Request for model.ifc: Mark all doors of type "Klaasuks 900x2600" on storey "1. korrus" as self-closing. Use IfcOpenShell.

First a look at what the model holds.

```python
import ifcopenshell
import ifcopenshell.util.element

model = ifcopenshell.open("model.ifc")
print(model.schema)
storey = next(s for s in model.by_type("IfcBuildingStorey") if s.Name == "1. korrus")
doors = [e for e in ifcopenshell.util.element.get_decomposition(storey) if e.is_a("IfcDoor")]
seen = {}
for e in doors:
    element_type = ifcopenshell.util.element.get_type(e)
    key = (element_type.Name if element_type != e and element_type else None, ifcopenshell.util.element.get_pset(e, "Pset_DoorCommon", "SelfClosing"))
    seen[key] = seen.get(key, 0) + 1
for (name, value), count in sorted(seen.items(), key=str):
    print(count, "x", name, "|", value)
```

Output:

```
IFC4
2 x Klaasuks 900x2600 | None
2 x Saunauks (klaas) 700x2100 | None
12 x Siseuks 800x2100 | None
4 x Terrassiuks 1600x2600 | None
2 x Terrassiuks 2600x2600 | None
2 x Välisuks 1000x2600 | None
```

```python
import ifcopenshell
import ifcopenshell.api.pset
import ifcopenshell.util.element

model = ifcopenshell.open("model.ifc")

storey = next(s for s in model.by_type("IfcBuildingStorey") if s.Name == "1. korrus")
doors = [e for e in ifcopenshell.util.element.get_decomposition(storey) if e.is_a("IfcDoor")]

count = 0
for e in doors:
    element_type = ifcopenshell.util.element.get_type(e)
    if element_type in (None, e) or element_type.Name != "Klaasuks 900x2600":
        continue
    # add_pset returns the element's existing set when there is one.
    pset = ifcopenshell.api.pset.add_pset(model, product=e, name="Pset_DoorCommon")
    ifcopenshell.api.pset.edit_pset(model, pset=pset, properties={"SelfClosing": True})
    count += 1

print(count, "doors updated")

model.write("model_v2.ifc")
```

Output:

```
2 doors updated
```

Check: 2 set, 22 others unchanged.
